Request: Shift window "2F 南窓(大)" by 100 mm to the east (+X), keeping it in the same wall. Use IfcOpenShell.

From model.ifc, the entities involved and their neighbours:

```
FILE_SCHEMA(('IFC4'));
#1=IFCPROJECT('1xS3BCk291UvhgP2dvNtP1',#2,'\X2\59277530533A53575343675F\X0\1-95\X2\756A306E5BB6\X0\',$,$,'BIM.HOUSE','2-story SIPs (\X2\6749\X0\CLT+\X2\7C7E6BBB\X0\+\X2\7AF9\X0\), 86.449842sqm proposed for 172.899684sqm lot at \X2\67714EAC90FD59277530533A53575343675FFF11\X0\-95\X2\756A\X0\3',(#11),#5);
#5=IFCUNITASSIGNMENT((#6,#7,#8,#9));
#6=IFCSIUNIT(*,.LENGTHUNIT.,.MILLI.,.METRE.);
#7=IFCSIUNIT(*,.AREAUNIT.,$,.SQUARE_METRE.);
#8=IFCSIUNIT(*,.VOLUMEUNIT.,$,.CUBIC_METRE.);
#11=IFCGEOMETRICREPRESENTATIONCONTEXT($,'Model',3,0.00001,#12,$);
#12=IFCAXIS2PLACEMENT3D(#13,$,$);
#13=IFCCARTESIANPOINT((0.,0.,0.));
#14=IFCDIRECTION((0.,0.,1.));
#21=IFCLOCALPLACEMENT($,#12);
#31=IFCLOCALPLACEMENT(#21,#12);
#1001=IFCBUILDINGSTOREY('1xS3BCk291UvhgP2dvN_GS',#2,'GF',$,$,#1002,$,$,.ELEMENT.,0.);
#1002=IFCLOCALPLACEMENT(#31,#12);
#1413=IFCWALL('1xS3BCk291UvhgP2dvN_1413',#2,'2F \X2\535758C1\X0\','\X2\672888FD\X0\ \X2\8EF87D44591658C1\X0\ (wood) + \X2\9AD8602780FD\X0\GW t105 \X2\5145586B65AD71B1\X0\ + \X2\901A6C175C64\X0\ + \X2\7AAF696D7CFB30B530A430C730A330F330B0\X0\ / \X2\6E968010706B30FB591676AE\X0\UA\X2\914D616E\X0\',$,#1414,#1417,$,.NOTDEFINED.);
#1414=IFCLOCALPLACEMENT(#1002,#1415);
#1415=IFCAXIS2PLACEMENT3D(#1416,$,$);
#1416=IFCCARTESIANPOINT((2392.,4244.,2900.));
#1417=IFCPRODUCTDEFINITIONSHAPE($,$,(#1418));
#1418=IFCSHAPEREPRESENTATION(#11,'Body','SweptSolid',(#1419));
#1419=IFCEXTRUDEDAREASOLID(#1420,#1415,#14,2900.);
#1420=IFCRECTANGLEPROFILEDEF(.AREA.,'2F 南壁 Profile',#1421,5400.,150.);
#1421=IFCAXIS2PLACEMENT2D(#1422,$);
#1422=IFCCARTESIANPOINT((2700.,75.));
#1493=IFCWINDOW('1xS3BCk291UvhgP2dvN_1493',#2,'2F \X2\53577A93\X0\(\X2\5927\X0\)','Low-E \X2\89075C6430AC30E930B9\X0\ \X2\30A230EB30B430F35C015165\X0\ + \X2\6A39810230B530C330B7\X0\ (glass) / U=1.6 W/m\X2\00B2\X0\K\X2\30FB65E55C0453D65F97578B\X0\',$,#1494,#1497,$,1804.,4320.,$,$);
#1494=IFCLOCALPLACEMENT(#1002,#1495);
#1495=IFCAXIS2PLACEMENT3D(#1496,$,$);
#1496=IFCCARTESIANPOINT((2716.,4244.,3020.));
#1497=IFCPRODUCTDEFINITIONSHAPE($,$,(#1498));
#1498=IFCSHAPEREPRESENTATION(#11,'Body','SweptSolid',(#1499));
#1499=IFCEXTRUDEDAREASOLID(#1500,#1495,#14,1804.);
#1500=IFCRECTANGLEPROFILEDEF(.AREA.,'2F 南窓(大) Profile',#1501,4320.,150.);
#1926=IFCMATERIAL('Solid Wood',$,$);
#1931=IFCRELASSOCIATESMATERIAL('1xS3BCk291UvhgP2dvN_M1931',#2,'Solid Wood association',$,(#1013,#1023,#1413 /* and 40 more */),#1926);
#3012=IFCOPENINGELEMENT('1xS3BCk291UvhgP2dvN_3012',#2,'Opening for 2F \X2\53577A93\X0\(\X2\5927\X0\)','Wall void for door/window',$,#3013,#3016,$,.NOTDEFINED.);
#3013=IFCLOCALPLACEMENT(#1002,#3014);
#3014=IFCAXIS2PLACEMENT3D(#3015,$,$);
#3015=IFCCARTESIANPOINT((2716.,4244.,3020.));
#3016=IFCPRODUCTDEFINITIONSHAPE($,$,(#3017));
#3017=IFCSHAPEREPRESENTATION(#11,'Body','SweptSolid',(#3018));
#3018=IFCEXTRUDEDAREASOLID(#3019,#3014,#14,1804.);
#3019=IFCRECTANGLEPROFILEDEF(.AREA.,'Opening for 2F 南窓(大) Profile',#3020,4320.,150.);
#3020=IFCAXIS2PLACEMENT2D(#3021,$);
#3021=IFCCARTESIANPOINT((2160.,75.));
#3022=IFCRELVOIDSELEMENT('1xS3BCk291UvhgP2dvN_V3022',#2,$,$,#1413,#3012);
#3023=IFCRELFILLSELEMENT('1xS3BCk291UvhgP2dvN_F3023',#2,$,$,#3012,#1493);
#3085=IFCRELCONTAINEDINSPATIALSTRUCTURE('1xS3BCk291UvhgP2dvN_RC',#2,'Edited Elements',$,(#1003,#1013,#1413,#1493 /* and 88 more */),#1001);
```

```python
import ifcopenshell
import ifcopenshell.api.geometry
import ifcopenshell.util.placement
import ifcopenshell.util.unit

model = ifcopenshell.open("model.ifc")
unit_scale = ifcopenshell.util.unit.calculate_unit_scale(model)

window = model.by_guid("1xS3BCk291UvhgP2dvN_1493")
opening = window.FillsVoids[0].RelatingOpeningElement
wall = opening.VoidsElements[0].RelatingBuildingElement

wall_matrix = ifcopenshell.util.placement.get_local_placement(wall.ObjectPlacement)
shift = wall_matrix[:3, 0] * 0.1 / unit_scale
before = ifcopenshell.util.placement.get_local_placement(window.ObjectPlacement)[:3, 3].copy()

# The window is not placed relative to its opening, so move both.
for product in (opening, window):
    matrix = ifcopenshell.util.placement.get_local_placement(product.ObjectPlacement)
    matrix[:3, 3] += shift
    ifcopenshell.api.geometry.edit_object_placement(model, product=product, matrix=matrix, is_si=False)

after = ifcopenshell.util.placement.get_local_placement(window.ObjectPlacement)[:3, 3]
print("window moved by", (after - before).round(3) + 0.0)

model.write("model_rev.ifc")
```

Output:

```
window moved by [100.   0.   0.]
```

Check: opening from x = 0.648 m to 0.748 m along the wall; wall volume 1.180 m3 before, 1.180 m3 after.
